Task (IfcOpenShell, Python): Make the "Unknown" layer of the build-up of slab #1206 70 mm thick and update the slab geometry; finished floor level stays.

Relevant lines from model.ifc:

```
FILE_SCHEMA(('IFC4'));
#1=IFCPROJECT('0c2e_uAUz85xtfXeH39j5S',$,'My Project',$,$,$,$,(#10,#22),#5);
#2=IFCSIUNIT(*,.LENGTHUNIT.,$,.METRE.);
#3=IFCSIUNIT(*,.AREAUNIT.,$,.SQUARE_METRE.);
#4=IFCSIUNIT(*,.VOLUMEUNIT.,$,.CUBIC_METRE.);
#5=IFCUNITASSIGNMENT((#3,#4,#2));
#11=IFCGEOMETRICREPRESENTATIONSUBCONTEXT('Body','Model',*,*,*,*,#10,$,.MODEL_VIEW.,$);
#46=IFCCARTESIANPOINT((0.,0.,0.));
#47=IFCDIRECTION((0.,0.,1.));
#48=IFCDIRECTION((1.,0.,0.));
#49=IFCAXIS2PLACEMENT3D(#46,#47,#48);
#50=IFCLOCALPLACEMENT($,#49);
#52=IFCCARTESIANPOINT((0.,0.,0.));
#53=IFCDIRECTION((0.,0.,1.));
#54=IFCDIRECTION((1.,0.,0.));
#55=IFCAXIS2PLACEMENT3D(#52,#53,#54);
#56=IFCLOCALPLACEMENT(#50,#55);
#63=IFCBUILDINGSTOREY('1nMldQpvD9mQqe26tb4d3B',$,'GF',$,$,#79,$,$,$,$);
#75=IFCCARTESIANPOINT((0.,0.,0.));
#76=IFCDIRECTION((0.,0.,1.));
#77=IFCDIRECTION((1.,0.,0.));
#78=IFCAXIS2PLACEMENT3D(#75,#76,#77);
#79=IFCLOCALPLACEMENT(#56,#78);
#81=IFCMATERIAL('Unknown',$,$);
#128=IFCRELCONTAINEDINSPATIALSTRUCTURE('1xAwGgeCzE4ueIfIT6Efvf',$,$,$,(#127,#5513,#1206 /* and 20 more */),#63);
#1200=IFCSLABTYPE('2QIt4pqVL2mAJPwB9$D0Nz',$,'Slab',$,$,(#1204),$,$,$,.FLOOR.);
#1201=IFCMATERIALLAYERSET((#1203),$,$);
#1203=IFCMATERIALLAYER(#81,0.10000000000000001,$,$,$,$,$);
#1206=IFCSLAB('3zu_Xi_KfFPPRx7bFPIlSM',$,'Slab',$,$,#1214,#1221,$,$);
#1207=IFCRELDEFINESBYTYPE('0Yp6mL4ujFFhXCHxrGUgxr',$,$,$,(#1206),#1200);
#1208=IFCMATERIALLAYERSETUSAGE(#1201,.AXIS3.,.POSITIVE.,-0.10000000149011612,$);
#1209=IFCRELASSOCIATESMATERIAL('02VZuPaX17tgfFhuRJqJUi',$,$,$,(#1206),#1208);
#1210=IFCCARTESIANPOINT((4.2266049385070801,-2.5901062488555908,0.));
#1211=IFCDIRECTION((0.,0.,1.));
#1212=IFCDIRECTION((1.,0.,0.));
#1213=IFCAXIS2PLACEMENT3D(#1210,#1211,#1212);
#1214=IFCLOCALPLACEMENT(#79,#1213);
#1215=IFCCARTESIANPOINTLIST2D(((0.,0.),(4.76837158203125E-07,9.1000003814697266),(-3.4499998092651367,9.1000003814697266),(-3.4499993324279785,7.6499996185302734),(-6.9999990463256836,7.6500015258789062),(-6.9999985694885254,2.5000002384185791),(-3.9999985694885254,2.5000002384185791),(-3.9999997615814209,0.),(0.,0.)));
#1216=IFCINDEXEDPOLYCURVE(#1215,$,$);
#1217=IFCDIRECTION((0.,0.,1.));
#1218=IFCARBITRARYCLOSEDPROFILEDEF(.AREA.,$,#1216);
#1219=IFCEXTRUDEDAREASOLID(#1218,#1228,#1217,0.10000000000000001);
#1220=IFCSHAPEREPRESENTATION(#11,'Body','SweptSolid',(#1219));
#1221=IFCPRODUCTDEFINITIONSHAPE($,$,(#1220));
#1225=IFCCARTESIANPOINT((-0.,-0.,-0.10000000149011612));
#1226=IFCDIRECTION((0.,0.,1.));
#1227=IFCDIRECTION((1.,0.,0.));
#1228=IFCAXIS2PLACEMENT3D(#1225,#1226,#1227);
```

```python
import ifcopenshell
import ifcopenshell.util.element
import ifcopenshell.util.representation
import ifcopenshell.util.unit

model = ifcopenshell.open("model.ifc")
unit_scale = ifcopenshell.util.unit.calculate_unit_scale(model)

layer_set = model.by_id(1201)
layer = next(l for l in layer_set.MaterialLayers if l.Material and l.Material.Name == "Unknown")
change = 0.07 / unit_scale - layer.LayerThickness
layer.LayerThickness += change

# Geometry does not follow the layer set by itself.
slabs = [e for e in ifcopenshell.util.element.get_elements_by_material(model, layer_set) if e.is_a("IfcSlab")]
for slab in sorted(slabs, key=lambda e: e.id()):
    body = ifcopenshell.util.representation.get_representation(slab, "Model", "Body")
    solid = body.Items[0]
    old_depth = solid.Depth
    solid.Depth += change
    # Extruded upwards: lower the start of the extrusion so the top stays.
    x, y, z = solid.Position.Location.Coordinates
    solid.Position.Location = model.createIfcCartesianPoint((x, y, z - change))
    print(slab.id(), f"{old_depth:g} -> {solid.Depth:g}")

# The layers are counted up from the underside, which has moved.
for usage in {ifcopenshell.util.element.get_material(slab) for slab in slabs}:
    usage.OffsetFromReferenceLine -= change

model.write("model_v2.ifc")
```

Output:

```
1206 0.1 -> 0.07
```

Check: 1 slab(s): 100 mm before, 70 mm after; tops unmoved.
